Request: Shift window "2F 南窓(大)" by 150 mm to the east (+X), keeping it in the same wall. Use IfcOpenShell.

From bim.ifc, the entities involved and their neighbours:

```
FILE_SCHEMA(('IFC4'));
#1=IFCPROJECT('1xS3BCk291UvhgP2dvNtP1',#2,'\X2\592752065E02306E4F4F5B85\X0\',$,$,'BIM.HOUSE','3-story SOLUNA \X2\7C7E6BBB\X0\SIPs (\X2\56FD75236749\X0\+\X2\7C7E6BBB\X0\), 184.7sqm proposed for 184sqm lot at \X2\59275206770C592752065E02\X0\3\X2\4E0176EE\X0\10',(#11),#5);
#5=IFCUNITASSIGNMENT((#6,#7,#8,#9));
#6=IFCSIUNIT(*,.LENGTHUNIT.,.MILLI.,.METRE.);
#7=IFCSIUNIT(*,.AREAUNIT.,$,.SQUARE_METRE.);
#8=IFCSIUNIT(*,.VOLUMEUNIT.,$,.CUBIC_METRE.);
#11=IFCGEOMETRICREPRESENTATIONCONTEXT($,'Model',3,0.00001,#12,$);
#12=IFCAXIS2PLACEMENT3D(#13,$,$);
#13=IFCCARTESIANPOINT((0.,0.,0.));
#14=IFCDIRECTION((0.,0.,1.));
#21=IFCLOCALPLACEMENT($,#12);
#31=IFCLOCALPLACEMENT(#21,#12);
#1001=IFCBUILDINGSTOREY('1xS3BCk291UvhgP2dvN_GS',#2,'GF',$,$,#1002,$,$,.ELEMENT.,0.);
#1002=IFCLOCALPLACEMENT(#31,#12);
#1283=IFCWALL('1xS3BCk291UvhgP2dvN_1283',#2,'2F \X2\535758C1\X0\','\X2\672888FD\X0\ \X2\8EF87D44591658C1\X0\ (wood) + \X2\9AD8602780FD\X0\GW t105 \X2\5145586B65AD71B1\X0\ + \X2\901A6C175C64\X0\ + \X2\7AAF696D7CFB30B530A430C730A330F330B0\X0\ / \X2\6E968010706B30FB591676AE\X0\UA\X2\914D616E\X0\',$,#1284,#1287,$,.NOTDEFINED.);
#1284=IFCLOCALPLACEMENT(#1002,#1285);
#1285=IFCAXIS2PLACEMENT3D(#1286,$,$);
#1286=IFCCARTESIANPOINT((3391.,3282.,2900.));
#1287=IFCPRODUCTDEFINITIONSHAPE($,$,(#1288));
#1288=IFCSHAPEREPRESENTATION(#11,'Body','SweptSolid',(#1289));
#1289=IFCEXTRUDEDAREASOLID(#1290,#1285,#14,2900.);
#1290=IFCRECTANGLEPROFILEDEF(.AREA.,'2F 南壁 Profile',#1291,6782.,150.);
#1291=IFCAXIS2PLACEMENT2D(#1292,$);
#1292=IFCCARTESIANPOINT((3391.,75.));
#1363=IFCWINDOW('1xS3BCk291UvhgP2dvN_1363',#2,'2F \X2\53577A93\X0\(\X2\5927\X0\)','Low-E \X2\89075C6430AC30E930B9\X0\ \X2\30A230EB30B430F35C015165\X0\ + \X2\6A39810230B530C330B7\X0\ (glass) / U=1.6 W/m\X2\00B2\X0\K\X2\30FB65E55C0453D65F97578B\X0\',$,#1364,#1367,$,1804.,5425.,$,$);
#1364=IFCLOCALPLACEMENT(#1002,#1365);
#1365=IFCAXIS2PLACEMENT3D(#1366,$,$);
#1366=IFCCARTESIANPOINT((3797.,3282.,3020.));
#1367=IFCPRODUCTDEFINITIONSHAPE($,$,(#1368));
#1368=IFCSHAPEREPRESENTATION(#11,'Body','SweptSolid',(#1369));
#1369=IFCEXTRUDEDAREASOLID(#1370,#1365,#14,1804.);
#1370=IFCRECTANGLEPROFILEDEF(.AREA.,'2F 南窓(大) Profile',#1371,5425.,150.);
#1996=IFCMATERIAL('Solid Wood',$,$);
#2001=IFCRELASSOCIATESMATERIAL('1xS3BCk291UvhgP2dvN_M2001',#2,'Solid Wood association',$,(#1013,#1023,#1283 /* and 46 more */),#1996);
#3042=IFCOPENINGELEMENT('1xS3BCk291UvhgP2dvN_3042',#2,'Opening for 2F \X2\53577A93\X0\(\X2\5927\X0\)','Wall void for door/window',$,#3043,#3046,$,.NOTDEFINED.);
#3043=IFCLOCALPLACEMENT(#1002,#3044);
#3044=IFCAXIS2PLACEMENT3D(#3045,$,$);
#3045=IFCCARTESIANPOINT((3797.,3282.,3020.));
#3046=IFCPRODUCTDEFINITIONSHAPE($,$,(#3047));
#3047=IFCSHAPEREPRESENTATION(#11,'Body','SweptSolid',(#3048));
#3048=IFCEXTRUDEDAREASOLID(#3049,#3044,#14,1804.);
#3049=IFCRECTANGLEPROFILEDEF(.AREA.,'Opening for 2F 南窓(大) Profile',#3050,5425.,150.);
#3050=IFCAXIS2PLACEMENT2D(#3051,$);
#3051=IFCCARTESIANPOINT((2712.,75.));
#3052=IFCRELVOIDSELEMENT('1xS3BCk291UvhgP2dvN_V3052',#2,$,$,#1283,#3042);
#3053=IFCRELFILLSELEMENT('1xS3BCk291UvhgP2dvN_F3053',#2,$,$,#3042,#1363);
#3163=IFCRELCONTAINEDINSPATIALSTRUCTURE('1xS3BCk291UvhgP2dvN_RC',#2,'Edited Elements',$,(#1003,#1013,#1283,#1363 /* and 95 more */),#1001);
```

```python
import ifcopenshell
import ifcopenshell.api.geometry
import ifcopenshell.util.placement
import ifcopenshell.util.unit

model = ifcopenshell.open("bim.ifc")
unit_scale = ifcopenshell.util.unit.calculate_unit_scale(model)

window = model.by_id(1363)
opening = window.FillsVoids[0].RelatingOpeningElement
wall = opening.VoidsElements[0].RelatingBuildingElement

wall_matrix = ifcopenshell.util.placement.get_local_placement(wall.ObjectPlacement)
shift = wall_matrix[:3, 0] * 0.15 / unit_scale
before = ifcopenshell.util.placement.get_local_placement(window.ObjectPlacement)[:3, 3].copy()

# The window is not placed relative to its opening, so move both.
for product in (opening, window):
    matrix = ifcopenshell.util.placement.get_local_placement(product.ObjectPlacement)
    matrix[:3, 3] += shift
    ifcopenshell.api.geometry.edit_object_placement(model, product=product, matrix=matrix, is_si=False)

after = ifcopenshell.util.placement.get_local_placement(window.ObjectPlacement)[:3, 3]
print("window moved by", (after - before).round(3) + 0.0)

model.write("bim_updated.ifc")
```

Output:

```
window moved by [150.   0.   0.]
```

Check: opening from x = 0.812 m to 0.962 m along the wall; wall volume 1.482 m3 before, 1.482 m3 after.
